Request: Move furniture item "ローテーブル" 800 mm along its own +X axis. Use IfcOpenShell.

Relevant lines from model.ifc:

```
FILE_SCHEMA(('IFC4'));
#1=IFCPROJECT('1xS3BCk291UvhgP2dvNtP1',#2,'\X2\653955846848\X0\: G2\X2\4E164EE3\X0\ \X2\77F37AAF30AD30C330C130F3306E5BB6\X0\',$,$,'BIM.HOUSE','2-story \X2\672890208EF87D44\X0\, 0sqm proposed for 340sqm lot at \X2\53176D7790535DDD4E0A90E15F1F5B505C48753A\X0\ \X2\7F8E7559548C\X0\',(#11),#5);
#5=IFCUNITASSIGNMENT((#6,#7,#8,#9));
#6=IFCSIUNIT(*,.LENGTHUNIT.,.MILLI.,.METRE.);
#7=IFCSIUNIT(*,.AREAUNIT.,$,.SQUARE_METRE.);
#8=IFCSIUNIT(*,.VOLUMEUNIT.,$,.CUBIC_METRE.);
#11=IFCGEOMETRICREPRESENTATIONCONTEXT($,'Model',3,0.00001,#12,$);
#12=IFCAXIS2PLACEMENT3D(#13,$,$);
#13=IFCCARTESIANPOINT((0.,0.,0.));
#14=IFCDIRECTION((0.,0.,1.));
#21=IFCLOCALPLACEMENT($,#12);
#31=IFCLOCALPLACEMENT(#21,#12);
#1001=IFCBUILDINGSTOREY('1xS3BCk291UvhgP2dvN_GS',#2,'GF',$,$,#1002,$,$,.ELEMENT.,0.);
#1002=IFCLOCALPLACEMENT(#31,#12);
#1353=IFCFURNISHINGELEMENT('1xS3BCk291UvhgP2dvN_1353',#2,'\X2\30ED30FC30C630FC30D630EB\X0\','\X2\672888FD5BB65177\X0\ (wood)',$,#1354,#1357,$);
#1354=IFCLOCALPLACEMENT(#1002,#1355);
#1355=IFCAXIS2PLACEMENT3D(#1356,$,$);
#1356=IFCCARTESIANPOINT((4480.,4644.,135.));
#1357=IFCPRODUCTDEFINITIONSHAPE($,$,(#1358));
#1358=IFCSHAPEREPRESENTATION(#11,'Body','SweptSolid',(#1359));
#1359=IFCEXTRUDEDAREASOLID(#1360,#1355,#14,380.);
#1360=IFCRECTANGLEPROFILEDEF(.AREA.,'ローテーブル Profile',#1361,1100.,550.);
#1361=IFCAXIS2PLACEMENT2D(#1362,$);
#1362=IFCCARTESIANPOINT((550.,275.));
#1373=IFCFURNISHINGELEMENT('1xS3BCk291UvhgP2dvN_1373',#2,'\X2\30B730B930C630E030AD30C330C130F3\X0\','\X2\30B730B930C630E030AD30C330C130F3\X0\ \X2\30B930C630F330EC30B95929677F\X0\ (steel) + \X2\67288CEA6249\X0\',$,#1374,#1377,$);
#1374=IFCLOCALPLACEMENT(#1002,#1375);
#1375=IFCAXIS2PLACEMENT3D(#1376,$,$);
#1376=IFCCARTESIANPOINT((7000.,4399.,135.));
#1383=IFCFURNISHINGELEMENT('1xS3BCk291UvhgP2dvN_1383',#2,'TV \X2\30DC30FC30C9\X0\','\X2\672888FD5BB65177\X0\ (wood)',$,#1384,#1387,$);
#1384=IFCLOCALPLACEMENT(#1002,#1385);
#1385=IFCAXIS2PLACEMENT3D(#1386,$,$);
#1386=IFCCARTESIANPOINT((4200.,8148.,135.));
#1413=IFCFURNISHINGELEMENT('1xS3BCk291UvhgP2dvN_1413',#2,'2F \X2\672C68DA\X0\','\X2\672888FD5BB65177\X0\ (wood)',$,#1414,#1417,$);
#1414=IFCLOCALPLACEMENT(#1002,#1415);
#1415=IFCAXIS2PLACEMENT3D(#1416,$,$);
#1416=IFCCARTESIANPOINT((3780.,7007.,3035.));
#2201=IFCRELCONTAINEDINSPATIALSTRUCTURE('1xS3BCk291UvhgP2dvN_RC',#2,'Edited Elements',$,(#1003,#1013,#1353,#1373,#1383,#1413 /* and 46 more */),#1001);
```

```python
import ifcopenshell
import ifcopenshell.api.geometry
import ifcopenshell.util.placement
import ifcopenshell.util.unit

model = ifcopenshell.open("model.ifc")
unit_scale = ifcopenshell.util.unit.calculate_unit_scale(model)

item = model.by_guid("1xS3BCk291UvhgP2dvN_1353")
matrix = ifcopenshell.util.placement.get_local_placement(item.ObjectPlacement)
matrix[:3, 3] += matrix[:3, 0] * 0.8 / unit_scale
ifcopenshell.api.geometry.edit_object_placement(model, product=item, matrix=matrix, is_si=False)

print(ifcopenshell.util.placement.get_local_placement(item.ObjectPlacement).round(3) + 0.0)

model.write("model_v2.ifc")
```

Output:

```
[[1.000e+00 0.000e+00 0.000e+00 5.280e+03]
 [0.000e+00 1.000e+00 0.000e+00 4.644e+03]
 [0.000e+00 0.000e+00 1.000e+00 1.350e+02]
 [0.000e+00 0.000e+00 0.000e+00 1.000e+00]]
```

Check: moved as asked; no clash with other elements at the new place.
